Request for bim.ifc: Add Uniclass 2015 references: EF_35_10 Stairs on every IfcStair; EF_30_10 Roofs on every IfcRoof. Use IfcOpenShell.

First a look at what the model holds.

```python
import ifcopenshell

model = ifcopenshell.open("bim.ifc")
print(model.schema)
print("classifications:", [c.Name for c in model.by_type("IfcClassification")])
for ifc_class in ("IfcDoor", "IfcRoof", "IfcStair", "IfcWall", "IfcWindow"):
    print(ifc_class, len(model.by_type(ifc_class)))
```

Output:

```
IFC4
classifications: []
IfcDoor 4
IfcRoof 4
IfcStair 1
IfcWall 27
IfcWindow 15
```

```python
import ifcopenshell
import ifcopenshell.api.classification

model = ifcopenshell.open("bim.ifc")

system = ifcopenshell.api.classification.add_classification(model, classification="Uniclass 2015")

codes = {
    "IfcStair": ("EF_35_10", "Stairs"),
    "IfcRoof": ("EF_30_10", "Roofs"),
}
for ifc_class, (code, name) in codes.items():
    products = model.by_type(ifc_class)
    ifcopenshell.api.classification.add_reference(
        model, products=products, classification=system, identification=code, name=name
    )
    print(code, len(products))

model.write("bim_updated.ifc")
```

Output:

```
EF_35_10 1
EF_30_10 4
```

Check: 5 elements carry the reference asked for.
